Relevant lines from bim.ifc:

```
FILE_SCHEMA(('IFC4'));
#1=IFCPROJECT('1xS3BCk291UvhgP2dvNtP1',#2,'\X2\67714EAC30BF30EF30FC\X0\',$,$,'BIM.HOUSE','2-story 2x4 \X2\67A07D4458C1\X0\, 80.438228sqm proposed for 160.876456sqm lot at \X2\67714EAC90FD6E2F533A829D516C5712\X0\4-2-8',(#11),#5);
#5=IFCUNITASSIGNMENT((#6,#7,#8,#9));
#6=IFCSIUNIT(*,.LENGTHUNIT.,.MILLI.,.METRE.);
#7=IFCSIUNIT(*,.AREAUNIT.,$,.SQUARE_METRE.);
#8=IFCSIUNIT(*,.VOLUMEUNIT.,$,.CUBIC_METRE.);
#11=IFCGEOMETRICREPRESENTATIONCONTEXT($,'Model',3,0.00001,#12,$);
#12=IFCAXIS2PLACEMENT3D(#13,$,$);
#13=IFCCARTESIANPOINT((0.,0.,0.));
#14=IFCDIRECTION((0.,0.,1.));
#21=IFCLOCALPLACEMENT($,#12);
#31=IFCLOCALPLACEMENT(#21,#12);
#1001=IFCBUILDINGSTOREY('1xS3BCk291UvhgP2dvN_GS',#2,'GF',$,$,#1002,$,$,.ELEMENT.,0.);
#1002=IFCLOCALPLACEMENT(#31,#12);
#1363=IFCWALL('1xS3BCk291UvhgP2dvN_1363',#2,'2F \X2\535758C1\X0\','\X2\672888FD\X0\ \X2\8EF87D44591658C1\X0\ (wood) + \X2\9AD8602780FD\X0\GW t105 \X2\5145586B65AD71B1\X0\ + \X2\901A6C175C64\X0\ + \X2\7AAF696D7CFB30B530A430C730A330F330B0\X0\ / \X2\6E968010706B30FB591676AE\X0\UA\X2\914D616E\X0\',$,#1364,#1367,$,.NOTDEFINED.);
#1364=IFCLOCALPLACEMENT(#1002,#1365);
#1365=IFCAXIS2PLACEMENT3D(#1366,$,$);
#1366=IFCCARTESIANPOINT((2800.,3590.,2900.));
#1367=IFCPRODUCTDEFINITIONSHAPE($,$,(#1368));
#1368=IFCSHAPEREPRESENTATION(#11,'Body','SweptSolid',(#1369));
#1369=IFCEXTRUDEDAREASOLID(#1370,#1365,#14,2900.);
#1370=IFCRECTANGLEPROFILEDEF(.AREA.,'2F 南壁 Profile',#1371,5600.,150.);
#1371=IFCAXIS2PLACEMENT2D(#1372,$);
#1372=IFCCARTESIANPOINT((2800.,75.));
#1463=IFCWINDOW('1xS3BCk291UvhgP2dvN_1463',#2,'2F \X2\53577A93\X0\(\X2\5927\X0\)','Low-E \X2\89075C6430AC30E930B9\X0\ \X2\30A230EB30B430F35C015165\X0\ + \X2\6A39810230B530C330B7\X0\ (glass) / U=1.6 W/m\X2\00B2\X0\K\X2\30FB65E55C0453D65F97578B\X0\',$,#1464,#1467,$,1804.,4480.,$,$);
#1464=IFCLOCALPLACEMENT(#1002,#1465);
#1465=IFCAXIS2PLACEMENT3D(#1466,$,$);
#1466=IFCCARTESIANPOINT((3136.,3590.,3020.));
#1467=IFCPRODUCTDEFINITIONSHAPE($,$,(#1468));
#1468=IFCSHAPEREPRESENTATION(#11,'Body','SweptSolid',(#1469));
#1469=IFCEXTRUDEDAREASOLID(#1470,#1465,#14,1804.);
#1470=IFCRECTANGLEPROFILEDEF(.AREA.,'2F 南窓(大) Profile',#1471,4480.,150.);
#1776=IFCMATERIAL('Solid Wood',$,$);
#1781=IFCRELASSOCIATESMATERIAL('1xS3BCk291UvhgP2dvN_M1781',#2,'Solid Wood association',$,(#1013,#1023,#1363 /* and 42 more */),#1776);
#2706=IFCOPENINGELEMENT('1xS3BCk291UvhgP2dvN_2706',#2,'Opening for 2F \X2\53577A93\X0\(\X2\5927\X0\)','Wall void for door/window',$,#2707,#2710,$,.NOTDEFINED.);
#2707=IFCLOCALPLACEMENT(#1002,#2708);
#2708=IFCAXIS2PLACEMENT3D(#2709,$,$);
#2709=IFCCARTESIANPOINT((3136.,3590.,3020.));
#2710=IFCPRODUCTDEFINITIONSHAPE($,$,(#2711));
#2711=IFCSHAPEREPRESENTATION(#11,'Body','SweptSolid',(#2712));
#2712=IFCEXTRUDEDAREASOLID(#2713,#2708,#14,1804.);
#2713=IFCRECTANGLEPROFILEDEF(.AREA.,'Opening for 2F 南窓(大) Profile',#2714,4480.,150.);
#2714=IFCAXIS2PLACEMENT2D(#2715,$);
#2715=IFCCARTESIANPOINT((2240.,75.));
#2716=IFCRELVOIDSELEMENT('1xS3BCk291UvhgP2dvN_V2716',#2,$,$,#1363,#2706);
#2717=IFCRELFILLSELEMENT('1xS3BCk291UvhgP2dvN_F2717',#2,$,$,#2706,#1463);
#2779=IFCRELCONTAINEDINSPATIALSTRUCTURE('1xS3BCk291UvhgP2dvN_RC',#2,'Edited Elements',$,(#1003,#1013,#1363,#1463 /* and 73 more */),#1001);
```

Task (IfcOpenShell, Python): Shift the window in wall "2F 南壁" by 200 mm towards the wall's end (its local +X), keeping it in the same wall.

```python
import ifcopenshell
import ifcopenshell.api.geometry
import ifcopenshell.util.placement
import ifcopenshell.util.unit

model = ifcopenshell.open("bim.ifc")
unit_scale = ifcopenshell.util.unit.calculate_unit_scale(model)

window = model.by_guid("1xS3BCk291UvhgP2dvN_1463")
opening = window.FillsVoids[0].RelatingOpeningElement
wall = opening.VoidsElements[0].RelatingBuildingElement

wall_matrix = ifcopenshell.util.placement.get_local_placement(wall.ObjectPlacement)
shift = wall_matrix[:3, 0] * 0.2 / unit_scale
before = ifcopenshell.util.placement.get_local_placement(window.ObjectPlacement)[:3, 3].copy()

# The window is not placed relative to its opening, so move both.
for product in (opening, window):
    matrix = ifcopenshell.util.placement.get_local_placement(product.ObjectPlacement)
    matrix[:3, 3] += shift
    ifcopenshell.api.geometry.edit_object_placement(model, product=product, matrix=matrix, is_si=False)

after = ifcopenshell.util.placement.get_local_placement(window.ObjectPlacement)[:3, 3]
print("window moved by", (after - before).round(3) + 0.0)

model.write("bim-out.ifc")
```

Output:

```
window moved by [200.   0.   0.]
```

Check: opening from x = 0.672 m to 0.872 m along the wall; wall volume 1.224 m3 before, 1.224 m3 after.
